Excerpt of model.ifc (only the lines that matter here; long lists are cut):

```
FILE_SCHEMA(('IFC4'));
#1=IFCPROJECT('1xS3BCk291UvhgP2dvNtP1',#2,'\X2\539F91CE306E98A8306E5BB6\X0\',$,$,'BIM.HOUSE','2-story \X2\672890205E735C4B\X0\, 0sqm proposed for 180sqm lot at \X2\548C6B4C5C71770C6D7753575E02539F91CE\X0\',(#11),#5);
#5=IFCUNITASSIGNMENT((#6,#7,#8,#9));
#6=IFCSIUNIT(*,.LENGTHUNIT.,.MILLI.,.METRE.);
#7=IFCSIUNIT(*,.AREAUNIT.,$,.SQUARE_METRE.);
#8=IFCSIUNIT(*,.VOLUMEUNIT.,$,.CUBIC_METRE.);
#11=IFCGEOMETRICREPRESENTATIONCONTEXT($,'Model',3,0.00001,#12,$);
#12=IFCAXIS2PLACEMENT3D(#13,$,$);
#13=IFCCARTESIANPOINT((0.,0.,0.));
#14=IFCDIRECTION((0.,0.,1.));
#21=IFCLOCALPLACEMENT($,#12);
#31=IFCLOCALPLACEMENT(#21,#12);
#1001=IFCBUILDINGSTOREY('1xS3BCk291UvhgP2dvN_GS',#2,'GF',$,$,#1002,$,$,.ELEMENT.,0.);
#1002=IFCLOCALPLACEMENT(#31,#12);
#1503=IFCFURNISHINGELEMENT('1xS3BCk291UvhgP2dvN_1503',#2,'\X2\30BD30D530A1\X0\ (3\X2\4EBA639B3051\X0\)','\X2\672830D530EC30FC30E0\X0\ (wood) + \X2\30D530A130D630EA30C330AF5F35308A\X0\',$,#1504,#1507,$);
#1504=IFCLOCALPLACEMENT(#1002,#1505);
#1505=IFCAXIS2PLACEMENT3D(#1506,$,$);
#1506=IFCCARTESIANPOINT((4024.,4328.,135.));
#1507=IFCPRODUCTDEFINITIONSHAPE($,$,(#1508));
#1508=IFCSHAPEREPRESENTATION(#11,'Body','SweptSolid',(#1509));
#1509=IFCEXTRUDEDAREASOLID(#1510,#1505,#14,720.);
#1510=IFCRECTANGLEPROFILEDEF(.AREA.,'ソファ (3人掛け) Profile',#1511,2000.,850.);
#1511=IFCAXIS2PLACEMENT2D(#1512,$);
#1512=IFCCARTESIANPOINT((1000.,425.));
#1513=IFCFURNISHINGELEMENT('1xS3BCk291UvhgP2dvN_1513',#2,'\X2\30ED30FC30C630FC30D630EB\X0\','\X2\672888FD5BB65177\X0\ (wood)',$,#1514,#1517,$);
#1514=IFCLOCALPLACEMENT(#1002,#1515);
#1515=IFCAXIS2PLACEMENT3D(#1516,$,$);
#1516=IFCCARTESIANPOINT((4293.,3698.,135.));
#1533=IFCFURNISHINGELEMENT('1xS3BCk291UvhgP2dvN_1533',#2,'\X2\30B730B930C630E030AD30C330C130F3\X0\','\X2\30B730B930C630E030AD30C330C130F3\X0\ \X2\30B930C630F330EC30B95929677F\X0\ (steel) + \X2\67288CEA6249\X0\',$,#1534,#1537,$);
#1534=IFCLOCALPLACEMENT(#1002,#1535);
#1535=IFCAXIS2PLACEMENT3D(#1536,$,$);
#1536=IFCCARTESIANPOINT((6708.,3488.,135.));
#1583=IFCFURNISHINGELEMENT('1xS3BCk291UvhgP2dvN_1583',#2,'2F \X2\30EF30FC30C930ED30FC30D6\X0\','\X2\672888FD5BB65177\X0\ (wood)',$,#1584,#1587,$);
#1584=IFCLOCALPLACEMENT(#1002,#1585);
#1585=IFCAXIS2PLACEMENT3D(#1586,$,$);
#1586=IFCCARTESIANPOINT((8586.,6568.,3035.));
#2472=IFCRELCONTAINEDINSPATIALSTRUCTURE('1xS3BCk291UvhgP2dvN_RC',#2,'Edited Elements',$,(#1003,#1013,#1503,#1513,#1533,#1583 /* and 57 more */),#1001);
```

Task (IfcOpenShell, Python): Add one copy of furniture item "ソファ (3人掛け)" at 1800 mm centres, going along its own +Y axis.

```python
import ifcopenshell
import ifcopenshell.api.geometry
import ifcopenshell.api.root
import ifcopenshell.util.element
import ifcopenshell.util.placement
import ifcopenshell.util.unit

model = ifcopenshell.open("model.ifc")
unit_scale = ifcopenshell.util.unit.calculate_unit_scale(model)


def reuse_history(source, copy):
    """copy_class also copies each property set's owner history, people and application; keep the originals."""
    for rel in copy.IsDefinedBy:
        if rel.is_a("IfcRelDefinesByProperties") and (history := rel.RelatingPropertyDefinition.OwnerHistory):
            rel.RelatingPropertyDefinition.OwnerHistory = source.OwnerHistory
            ifcopenshell.util.element.remove_deep2(model, history)


source = model.by_guid("1xS3BCk291UvhgP2dvN_1503")
base = ifcopenshell.util.placement.get_local_placement(source.ObjectPlacement)
step = base[:3, 1] * 1.8 / unit_scale

for i in range(1, 2):
    copy = ifcopenshell.api.root.copy_class(model, product=source)
    copy.Representation = ifcopenshell.util.element.copy_deep(
        model, source.Representation, exclude=["IfcGeometricRepresentationContext", "IfcRepresentationMap"]
    )
    reuse_history(source, copy)
    matrix = base.copy()
    matrix[:3, 3] += i * step
    print("added at", matrix[:3, 3].round(3) + 0.0)
    ifcopenshell.api.geometry.edit_object_placement(model, product=copy, matrix=matrix, is_si=False)

model.write("model_rev.ifc")
```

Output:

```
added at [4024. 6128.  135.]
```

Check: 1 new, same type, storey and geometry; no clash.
